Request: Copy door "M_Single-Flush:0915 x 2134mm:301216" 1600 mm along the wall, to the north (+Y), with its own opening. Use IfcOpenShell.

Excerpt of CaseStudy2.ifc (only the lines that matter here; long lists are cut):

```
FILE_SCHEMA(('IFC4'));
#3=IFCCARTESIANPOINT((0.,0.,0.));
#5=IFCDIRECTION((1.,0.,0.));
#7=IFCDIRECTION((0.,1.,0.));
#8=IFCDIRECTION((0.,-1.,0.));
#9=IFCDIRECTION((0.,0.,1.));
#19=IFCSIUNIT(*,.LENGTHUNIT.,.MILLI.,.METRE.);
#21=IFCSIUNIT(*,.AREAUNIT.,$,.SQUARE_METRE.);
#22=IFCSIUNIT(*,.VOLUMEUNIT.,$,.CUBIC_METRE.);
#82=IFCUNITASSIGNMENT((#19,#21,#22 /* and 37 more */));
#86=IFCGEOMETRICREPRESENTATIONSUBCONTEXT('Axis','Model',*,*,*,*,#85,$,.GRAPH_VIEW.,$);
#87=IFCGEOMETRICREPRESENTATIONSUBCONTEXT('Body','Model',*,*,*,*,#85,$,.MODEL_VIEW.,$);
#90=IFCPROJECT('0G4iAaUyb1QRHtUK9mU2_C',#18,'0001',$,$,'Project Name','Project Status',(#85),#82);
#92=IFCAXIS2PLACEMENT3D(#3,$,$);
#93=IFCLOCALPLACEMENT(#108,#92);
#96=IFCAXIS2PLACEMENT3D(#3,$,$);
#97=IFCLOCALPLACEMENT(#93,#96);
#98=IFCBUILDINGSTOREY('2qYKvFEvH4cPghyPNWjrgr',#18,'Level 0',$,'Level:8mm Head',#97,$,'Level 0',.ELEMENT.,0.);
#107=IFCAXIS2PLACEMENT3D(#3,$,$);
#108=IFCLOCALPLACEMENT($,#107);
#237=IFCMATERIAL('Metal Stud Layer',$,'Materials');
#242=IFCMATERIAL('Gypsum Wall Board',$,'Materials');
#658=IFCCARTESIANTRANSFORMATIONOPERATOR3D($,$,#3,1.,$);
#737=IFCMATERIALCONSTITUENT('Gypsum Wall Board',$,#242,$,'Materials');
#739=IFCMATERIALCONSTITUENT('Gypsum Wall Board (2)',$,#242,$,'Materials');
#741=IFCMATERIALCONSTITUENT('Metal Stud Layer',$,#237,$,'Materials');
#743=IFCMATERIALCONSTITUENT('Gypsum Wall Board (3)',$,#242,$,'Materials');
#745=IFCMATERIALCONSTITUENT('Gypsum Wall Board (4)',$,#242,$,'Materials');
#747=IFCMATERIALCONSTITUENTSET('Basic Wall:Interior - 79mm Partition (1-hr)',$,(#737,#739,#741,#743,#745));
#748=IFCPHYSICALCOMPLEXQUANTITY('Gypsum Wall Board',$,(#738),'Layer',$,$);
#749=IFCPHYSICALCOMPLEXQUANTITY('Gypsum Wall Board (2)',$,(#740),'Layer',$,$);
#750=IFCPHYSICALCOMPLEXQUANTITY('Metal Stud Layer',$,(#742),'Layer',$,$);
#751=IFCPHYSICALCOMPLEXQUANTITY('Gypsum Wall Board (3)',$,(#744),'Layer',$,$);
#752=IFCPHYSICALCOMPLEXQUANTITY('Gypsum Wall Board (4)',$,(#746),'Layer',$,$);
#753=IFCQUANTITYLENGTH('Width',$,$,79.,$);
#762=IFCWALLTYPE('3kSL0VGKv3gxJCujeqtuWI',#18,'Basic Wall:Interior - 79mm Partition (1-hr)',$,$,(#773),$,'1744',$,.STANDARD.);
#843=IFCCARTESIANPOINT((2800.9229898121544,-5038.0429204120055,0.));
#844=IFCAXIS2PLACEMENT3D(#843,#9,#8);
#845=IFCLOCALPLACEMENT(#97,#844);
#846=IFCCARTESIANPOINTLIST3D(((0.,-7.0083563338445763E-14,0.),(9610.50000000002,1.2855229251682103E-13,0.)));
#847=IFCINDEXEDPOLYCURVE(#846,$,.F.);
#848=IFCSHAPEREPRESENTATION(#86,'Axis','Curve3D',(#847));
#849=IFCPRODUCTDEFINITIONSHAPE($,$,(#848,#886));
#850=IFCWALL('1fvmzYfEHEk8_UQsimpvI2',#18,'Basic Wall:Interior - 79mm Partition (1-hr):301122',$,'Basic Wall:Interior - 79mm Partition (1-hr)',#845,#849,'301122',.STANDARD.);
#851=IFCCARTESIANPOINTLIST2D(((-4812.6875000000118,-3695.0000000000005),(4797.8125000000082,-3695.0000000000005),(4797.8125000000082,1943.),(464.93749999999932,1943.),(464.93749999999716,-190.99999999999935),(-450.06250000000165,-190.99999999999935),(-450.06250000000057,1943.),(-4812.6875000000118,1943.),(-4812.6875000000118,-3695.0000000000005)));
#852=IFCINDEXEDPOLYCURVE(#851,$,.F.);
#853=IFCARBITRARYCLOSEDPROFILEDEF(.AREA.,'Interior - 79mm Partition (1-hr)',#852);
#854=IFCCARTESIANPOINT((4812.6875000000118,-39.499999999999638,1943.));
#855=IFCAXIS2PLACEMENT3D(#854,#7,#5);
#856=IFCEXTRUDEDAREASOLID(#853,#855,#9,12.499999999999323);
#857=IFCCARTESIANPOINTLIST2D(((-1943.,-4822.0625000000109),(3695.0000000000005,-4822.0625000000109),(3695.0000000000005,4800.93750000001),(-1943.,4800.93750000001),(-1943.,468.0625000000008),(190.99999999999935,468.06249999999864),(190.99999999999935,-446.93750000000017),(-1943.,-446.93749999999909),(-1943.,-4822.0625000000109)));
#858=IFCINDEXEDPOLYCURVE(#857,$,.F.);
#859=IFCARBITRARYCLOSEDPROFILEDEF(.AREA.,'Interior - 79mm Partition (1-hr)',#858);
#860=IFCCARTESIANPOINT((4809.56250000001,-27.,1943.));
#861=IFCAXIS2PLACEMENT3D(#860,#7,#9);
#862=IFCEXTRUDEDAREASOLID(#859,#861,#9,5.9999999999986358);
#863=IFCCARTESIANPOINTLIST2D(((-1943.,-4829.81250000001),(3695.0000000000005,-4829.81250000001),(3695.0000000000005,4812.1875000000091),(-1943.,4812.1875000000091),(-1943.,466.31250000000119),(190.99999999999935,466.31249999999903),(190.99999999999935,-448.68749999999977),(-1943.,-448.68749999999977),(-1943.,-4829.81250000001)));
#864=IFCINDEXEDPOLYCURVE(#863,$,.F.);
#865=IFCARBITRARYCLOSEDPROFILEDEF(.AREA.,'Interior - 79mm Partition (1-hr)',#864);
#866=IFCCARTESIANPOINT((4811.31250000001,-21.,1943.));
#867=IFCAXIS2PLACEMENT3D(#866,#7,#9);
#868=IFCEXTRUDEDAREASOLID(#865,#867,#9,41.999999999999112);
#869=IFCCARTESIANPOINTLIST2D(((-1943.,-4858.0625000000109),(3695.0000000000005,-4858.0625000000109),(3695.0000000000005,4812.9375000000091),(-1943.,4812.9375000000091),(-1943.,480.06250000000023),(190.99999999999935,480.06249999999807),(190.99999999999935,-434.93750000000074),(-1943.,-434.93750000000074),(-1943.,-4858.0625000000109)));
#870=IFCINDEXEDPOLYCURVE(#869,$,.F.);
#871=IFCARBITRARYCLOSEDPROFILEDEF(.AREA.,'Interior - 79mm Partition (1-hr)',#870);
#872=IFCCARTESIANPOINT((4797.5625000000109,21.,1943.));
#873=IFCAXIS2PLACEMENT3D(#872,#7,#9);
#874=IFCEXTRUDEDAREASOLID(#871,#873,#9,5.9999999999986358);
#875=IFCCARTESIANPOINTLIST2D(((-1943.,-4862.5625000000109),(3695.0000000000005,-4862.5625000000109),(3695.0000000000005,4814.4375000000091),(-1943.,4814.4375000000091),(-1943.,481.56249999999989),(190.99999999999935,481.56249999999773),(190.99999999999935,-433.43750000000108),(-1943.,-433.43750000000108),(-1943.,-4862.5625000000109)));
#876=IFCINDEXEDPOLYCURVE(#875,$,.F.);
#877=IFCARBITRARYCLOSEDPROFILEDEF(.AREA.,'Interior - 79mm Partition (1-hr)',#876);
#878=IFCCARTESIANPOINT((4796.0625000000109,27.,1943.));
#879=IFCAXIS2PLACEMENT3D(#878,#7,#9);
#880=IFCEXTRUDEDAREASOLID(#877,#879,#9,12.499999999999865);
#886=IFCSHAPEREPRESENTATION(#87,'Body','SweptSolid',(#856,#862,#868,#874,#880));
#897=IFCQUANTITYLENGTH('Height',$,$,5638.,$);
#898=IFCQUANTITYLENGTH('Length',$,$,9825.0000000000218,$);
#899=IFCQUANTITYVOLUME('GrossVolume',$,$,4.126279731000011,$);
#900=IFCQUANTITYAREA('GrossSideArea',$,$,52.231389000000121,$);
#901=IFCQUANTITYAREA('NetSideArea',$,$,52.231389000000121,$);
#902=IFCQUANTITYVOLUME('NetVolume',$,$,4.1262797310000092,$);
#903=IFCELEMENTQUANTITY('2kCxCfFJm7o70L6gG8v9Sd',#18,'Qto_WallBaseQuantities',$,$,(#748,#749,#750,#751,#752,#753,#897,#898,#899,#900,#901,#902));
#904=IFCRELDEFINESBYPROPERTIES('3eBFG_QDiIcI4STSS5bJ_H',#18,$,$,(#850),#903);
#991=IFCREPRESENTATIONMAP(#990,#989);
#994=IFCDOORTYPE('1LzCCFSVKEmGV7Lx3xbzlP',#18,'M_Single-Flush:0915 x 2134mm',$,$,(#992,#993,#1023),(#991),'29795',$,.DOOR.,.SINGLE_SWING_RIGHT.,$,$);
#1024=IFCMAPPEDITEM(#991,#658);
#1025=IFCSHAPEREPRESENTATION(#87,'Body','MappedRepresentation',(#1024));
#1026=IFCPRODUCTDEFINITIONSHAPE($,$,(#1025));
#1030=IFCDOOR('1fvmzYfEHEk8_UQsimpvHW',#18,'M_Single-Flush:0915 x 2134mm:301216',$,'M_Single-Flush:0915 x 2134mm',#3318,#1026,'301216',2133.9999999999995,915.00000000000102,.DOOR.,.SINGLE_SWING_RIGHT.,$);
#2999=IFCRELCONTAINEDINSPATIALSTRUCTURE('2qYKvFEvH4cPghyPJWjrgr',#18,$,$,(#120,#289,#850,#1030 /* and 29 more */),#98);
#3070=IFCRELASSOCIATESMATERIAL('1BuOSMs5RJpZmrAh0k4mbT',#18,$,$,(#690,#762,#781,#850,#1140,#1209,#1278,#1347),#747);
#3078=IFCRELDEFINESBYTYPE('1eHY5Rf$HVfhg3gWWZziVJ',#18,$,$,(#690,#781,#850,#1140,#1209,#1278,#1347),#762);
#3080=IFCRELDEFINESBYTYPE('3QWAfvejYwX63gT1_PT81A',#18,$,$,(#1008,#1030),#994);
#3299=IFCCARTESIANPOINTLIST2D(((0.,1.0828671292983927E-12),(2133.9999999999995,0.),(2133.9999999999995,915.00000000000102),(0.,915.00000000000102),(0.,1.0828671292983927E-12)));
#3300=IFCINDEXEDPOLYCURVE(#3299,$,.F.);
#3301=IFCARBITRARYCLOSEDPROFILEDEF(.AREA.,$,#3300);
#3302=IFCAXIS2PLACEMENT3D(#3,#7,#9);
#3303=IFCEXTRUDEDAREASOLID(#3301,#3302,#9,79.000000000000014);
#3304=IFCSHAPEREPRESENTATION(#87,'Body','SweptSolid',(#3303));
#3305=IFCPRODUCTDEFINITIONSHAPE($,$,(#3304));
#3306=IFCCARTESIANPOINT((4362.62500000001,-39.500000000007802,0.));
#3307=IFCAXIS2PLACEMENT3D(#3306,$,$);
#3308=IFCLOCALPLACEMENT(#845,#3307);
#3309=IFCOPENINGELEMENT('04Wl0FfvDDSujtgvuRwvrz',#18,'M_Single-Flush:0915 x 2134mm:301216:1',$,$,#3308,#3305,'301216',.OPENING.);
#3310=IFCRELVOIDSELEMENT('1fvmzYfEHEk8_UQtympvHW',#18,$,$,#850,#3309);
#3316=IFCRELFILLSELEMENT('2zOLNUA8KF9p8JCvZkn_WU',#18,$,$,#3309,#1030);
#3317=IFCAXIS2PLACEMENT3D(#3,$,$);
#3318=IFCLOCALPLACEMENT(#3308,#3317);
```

```python
import ifcopenshell
import ifcopenshell.api.feature
import ifcopenshell.api.geometry
import ifcopenshell.api.pset
import ifcopenshell.api.root
import ifcopenshell.geom
import ifcopenshell.util.element
import ifcopenshell.util.placement
import ifcopenshell.util.shape
import ifcopenshell.util.unit

model = ifcopenshell.open("CaseStudy2.ifc")
area_scale = ifcopenshell.util.unit.calculate_unit_scale(model, "AREAUNIT")
volume_scale = ifcopenshell.util.unit.calculate_unit_scale(model, "VOLUMEUNIT")
settings = ifcopenshell.geom.settings()


def volume(element):
    """Net volume in cubic metres, openings subtracted."""
    shape = ifcopenshell.geom.create_shape(settings, element)
    return ifcopenshell.util.shape.get_volume(shape.geometry)


def reuse_history(source, copy):
    """copy_class also copies each property set's owner history, people and application; keep the originals."""
    for rel in copy.IsDefinedBy:
        if rel.is_a("IfcRelDefinesByProperties") and (history := rel.RelatingPropertyDefinition.OwnerHistory):
            rel.RelatingPropertyDefinition.OwnerHistory = source.OwnerHistory
            ifcopenshell.util.element.remove_deep2(model, history)


door = model.by_guid("1fvmzYfEHEk8_UQsimpvHW")
opening = door.FillsVoids[0].RelatingOpeningElement
wall = opening.VoidsElements[0].RelatingBuildingElement
before = volume(wall)
shift = ifcopenshell.util.placement.get_local_placement(wall.ObjectPlacement)[:3, 0] * -1600.0

# copy_class copies the void relationship, type, container and properties, but no geometry.
new_opening = ifcopenshell.api.root.copy_class(model, product=opening)
new_opening.Representation = ifcopenshell.util.element.copy_deep(
    model, opening.Representation, exclude=["IfcGeometricRepresentationContext", "IfcRepresentationMap"]
)
new_opening.Name = "M_Single-Flush:0915 x 2134mm"
new_opening.Tag = None
reuse_history(opening, new_opening)
new_door = ifcopenshell.api.root.copy_class(model, product=door)
new_door.Representation = ifcopenshell.util.element.copy_deep(
    model, door.Representation, exclude=["IfcGeometricRepresentationContext", "IfcRepresentationMap"]
)
new_door.Name = "M_Single-Flush:0915 x 2134mm"
new_door.Tag = None
reuse_history(door, new_door)
ifcopenshell.api.feature.add_filling(model, opening=new_opening, element=new_door)

for old, new in ((opening, new_opening), (door, new_door)):
    matrix = ifcopenshell.util.placement.get_local_placement(old.ObjectPlacement)
    matrix[:3, 3] += shift
    ifcopenshell.api.geometry.edit_object_placement(model, product=new, matrix=matrix, is_si=False)

after = volume(wall)
thickness = 0.079  # wall thickness in metres

# Update the wall's stored quantities.
qto = model.by_id(ifcopenshell.util.element.get_pset(wall, "Qto_WallBaseQuantities", should_inherit=False)["id"])
ifcopenshell.api.pset.edit_qto(model, qto=qto, properties={
    "NetSideArea": after / thickness / area_scale,
    "NetVolume": after / volume_scale,
})

print(f"wall volume {before:.3f} -> {after:.3f} m3")

model.write("CaseStudy2_updated.ifc")
```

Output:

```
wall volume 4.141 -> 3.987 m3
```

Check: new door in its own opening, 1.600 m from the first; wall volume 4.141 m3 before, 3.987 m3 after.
